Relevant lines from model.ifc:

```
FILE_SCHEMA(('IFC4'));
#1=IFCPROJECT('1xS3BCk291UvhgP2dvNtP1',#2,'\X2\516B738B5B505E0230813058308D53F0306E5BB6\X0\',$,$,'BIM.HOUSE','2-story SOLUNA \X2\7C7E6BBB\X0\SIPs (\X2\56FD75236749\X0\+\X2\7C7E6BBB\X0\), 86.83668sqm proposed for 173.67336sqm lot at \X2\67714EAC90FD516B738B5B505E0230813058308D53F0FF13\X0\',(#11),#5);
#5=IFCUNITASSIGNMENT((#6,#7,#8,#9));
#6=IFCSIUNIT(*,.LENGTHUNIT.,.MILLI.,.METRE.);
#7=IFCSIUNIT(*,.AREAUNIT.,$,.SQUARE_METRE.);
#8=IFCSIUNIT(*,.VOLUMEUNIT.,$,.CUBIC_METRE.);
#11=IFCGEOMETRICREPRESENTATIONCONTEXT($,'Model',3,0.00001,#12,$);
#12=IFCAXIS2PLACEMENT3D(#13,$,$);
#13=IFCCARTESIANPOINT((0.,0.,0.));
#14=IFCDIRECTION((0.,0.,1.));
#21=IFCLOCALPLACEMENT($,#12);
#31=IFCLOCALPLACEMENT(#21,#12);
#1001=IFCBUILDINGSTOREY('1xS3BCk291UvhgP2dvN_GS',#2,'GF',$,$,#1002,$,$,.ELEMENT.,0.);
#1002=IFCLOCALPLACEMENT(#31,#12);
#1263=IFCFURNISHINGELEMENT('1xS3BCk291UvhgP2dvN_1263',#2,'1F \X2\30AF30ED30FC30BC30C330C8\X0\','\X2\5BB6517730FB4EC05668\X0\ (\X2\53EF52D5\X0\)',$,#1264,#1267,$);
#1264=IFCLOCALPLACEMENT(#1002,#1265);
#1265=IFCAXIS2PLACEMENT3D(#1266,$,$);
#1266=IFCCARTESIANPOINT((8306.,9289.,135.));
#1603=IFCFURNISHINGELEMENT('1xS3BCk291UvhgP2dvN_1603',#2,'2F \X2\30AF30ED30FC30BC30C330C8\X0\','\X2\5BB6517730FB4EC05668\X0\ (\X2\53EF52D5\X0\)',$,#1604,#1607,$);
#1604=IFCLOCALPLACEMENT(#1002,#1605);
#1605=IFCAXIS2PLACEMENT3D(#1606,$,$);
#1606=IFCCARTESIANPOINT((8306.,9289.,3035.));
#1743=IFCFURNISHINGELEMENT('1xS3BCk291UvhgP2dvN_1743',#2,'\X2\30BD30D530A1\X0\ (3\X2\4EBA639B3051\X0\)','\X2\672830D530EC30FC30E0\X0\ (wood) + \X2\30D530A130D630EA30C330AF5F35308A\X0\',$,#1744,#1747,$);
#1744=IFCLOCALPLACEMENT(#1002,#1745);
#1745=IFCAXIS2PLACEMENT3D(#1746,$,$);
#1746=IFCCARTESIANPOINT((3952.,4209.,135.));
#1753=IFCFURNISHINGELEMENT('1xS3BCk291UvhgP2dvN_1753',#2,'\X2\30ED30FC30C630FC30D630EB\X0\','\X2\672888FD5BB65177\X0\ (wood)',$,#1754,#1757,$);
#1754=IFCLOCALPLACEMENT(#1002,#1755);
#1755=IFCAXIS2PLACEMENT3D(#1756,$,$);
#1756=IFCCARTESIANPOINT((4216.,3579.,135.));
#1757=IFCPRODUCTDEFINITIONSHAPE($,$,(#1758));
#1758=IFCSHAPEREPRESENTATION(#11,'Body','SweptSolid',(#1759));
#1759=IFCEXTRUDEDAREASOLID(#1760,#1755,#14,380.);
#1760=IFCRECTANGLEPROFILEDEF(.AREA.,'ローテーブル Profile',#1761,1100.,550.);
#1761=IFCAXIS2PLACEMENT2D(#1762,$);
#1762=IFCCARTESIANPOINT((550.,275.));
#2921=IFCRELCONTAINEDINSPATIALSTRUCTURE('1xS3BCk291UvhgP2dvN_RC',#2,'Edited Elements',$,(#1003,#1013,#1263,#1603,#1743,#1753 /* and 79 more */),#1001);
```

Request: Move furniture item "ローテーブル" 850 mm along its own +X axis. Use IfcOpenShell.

```python
import ifcopenshell
import ifcopenshell.api.geometry
import ifcopenshell.util.placement
import ifcopenshell.util.unit

model = ifcopenshell.open("model.ifc")
unit_scale = ifcopenshell.util.unit.calculate_unit_scale(model)

item = model.by_guid("1xS3BCk291UvhgP2dvN_1753")
matrix = ifcopenshell.util.placement.get_local_placement(item.ObjectPlacement)
matrix[:3, 3] += matrix[:3, 0] * 0.85 / unit_scale
ifcopenshell.api.geometry.edit_object_placement(model, product=item, matrix=matrix, is_si=False)

print(ifcopenshell.util.placement.get_local_placement(item.ObjectPlacement).round(3) + 0.0)

model.write("model-out.ifc")
```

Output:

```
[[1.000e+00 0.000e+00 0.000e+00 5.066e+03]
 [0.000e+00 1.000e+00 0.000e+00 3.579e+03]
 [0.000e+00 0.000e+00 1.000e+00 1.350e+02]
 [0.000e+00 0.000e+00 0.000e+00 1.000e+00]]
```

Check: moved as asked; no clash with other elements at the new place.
